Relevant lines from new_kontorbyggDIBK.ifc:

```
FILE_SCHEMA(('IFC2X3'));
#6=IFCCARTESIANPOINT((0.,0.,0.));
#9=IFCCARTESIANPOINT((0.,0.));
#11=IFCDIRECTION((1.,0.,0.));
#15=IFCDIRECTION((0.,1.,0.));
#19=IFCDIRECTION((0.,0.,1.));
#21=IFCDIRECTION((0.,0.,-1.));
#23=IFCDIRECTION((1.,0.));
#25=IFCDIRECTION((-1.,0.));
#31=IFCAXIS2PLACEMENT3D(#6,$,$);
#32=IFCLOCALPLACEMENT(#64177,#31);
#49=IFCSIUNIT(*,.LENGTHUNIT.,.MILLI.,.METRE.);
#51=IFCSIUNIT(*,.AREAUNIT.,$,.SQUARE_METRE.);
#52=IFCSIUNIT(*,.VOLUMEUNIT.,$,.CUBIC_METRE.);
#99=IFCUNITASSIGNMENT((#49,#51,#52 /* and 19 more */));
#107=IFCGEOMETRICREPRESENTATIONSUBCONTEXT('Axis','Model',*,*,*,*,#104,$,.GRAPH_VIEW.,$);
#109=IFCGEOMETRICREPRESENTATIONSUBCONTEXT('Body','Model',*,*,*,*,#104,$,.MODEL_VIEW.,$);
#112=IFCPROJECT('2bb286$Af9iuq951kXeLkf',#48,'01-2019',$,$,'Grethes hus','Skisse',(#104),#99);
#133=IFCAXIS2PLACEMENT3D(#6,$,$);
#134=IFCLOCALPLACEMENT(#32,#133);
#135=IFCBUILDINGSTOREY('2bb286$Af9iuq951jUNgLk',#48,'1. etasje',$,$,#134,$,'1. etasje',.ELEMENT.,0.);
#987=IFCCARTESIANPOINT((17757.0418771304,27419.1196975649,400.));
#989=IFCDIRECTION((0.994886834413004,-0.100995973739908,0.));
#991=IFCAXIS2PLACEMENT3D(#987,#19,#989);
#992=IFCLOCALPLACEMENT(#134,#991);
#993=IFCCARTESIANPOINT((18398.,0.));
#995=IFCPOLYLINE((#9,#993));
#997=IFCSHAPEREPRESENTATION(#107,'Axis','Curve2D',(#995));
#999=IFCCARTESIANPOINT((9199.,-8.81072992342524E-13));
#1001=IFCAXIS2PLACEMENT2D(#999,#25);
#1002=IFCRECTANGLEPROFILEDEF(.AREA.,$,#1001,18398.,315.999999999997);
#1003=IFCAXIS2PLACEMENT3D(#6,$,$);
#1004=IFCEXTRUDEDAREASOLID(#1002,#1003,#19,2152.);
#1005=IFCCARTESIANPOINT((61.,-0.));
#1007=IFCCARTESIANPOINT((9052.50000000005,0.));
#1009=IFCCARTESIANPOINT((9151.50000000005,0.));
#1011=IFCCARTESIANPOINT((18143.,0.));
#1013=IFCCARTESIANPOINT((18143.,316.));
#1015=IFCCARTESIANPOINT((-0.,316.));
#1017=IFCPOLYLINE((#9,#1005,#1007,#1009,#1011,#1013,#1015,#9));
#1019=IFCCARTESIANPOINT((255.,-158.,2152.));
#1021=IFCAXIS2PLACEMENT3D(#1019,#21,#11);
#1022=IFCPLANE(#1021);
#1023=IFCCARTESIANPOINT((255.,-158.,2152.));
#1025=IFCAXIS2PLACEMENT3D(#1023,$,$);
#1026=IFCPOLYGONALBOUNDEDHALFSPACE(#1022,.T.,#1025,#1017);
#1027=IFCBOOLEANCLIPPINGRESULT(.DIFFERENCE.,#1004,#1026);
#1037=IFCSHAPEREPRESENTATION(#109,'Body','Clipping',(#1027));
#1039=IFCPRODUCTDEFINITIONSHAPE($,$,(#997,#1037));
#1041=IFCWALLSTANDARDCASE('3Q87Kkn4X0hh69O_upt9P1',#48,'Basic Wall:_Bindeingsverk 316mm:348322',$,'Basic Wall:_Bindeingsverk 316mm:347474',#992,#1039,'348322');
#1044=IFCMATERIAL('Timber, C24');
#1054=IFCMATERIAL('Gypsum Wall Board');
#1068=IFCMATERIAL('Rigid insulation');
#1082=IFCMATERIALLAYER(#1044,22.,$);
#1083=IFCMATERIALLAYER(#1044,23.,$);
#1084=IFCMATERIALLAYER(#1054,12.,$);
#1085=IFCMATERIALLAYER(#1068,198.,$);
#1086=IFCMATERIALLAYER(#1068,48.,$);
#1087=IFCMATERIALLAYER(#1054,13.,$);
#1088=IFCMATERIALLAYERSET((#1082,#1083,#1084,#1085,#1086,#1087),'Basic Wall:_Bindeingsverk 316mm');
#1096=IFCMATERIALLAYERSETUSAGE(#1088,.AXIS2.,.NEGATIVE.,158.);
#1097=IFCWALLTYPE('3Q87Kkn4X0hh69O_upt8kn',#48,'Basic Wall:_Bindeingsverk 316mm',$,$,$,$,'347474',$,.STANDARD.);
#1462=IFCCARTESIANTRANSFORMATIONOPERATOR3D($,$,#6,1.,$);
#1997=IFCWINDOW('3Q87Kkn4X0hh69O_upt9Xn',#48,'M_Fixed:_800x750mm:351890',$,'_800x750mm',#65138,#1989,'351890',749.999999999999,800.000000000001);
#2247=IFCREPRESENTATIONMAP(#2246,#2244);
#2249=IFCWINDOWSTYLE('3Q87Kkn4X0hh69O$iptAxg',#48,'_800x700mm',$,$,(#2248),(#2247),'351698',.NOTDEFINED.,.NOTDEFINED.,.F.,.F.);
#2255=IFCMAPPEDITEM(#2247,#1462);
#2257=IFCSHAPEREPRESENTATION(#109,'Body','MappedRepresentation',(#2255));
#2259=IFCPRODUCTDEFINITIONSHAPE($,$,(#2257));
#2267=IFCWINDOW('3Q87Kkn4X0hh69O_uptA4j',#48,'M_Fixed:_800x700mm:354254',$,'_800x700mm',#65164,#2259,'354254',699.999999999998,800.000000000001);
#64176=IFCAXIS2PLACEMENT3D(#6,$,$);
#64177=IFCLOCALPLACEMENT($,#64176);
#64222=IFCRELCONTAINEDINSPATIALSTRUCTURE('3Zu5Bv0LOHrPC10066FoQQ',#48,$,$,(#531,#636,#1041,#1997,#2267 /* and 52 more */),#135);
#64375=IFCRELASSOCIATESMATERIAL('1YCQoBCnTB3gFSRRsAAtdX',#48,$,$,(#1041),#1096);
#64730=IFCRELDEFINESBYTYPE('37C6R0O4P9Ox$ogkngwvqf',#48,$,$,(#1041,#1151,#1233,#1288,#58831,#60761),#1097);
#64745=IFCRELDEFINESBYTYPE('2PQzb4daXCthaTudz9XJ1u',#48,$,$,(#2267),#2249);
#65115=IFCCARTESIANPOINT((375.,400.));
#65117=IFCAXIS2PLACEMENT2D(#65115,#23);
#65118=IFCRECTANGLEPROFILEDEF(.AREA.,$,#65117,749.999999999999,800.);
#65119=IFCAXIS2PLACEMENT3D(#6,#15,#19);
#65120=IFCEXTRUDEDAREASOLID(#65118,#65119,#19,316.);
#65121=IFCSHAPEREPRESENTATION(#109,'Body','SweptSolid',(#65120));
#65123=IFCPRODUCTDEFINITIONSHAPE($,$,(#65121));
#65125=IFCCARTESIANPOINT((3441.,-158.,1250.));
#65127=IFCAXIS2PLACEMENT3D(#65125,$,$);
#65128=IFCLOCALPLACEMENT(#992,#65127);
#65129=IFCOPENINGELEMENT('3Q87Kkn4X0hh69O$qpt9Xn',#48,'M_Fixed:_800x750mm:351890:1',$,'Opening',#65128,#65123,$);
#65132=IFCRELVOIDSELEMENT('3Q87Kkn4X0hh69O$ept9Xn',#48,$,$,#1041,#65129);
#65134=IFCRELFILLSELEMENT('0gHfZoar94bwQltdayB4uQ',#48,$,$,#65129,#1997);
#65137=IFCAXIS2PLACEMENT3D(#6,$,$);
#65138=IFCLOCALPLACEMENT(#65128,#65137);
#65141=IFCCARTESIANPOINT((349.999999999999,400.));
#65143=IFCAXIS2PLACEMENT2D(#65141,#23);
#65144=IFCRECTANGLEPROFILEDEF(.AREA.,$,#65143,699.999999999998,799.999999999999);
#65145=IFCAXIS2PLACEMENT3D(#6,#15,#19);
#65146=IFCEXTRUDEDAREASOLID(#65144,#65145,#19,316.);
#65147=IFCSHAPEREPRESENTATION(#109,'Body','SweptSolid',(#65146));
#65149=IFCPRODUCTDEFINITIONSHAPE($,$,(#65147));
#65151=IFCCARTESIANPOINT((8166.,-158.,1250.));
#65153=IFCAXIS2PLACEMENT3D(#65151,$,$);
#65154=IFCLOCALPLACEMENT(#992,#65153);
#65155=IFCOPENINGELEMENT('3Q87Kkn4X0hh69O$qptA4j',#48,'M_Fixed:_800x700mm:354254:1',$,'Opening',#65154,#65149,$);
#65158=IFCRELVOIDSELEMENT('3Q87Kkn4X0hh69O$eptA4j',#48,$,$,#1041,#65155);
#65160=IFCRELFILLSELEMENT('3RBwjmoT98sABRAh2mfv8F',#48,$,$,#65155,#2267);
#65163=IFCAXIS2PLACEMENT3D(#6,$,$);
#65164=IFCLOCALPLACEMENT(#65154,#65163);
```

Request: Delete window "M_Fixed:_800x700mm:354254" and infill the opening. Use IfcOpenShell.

```python
import ifcopenshell
import ifcopenshell.api.feature
import ifcopenshell.api.root
import ifcopenshell.geom
import ifcopenshell.util.shape

model = ifcopenshell.open("new_kontorbyggDIBK.ifc")
settings = ifcopenshell.geom.settings()


def volume(element):
    """Net volume in cubic metres, openings subtracted."""
    shape = ifcopenshell.geom.create_shape(settings, element)
    return ifcopenshell.util.shape.get_volume(shape.geometry)


window = model.by_id(2267)
opening = window.FillsVoids[0].RelatingOpeningElement
wall = opening.VoidsElements[0].RelatingBuildingElement
before = volume(wall)

ifcopenshell.api.root.remove_product(model, product=window)
ifcopenshell.api.feature.remove_feature(model, feature=opening)

after = volume(wall)

print(f"wall volume {before:.3f} -> {after:.3f} m3")

model.write("new_kontorbyggDIBK_updated.ifc")
```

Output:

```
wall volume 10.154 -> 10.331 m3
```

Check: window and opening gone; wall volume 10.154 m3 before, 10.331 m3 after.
